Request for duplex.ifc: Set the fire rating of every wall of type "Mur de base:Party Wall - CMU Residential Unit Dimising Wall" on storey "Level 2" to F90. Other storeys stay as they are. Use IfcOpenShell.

First a look at what the model holds.

```python
import ifcopenshell
import ifcopenshell.util.element

model = ifcopenshell.open("duplex.ifc")
print(model.schema)
storey = next(s for s in model.by_type("IfcBuildingStorey") if s.Name == "Level 2")
walls = [e for e in ifcopenshell.util.element.get_decomposition(storey) if e.is_a("IfcWall")]
seen = {}
for e in walls:
    element_type = ifcopenshell.util.element.get_type(e)
    key = (element_type.Name if element_type != e and element_type else None, ifcopenshell.util.element.get_pset(e, "Pset_WallCommon", "FireRating"))
    seen[key] = seen.get(key, 0) + 1
for (name, value), count in sorted(seen.items(), key=str):
    print(count, "x", name, "|", value)
```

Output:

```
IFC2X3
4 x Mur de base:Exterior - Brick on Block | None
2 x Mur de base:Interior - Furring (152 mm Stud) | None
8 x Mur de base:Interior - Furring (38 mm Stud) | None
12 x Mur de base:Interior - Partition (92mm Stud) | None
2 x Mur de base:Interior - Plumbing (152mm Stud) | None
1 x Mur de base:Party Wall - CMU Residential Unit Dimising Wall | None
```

```python
import ifcopenshell
import ifcopenshell.api.pset
import ifcopenshell.util.element

model = ifcopenshell.open("duplex.ifc")

storey = next(s for s in model.by_type("IfcBuildingStorey") if s.Name == "Level 2")
walls = [e for e in ifcopenshell.util.element.get_decomposition(storey) if e.is_a("IfcWall")]

count = 0
for e in walls:
    element_type = ifcopenshell.util.element.get_type(e)
    if element_type in (None, e) or element_type.Name != "Mur de base:Party Wall - CMU Residential Unit Dimising Wall":
        continue
    # add_pset returns the element's existing set when there is one.
    pset = ifcopenshell.api.pset.add_pset(model, product=e, name="Pset_WallCommon")
    ifcopenshell.api.pset.edit_pset(model, pset=pset, properties={"FireRating": "F90"})
    count += 1

print(count, "walls updated")

model.write("duplex-out.ifc")
```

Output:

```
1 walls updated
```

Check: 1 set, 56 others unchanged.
